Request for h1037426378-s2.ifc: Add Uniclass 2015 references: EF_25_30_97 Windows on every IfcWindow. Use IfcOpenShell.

First a look at what the model holds.

```python
import ifcopenshell

model = ifcopenshell.open("h1037426378-s2.ifc")
print(model.schema)
print("classifications:", [c.Name for c in model.by_type("IfcClassification")])
for ifc_class in ("IfcDoor", "IfcRoof", "IfcStair", "IfcWall", "IfcWindow"):
    print(ifc_class, len(model.by_type(ifc_class)))
```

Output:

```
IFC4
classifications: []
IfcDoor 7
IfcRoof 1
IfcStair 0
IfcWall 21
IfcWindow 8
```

```python
import ifcopenshell
import ifcopenshell.api.classification

model = ifcopenshell.open("h1037426378-s2.ifc")

system = ifcopenshell.api.classification.add_classification(model, classification="Uniclass 2015")

codes = {
    "IfcWindow": ("EF_25_30_97", "Windows"),
}
for ifc_class, (code, name) in codes.items():
    products = model.by_type(ifc_class)
    ifcopenshell.api.classification.add_reference(
        model, products=products, classification=system, identification=code, name=name
    )
    print(code, len(products))

model.write("h1037426378-s2_edited.ifc")
```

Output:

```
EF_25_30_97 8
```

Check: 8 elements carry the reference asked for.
